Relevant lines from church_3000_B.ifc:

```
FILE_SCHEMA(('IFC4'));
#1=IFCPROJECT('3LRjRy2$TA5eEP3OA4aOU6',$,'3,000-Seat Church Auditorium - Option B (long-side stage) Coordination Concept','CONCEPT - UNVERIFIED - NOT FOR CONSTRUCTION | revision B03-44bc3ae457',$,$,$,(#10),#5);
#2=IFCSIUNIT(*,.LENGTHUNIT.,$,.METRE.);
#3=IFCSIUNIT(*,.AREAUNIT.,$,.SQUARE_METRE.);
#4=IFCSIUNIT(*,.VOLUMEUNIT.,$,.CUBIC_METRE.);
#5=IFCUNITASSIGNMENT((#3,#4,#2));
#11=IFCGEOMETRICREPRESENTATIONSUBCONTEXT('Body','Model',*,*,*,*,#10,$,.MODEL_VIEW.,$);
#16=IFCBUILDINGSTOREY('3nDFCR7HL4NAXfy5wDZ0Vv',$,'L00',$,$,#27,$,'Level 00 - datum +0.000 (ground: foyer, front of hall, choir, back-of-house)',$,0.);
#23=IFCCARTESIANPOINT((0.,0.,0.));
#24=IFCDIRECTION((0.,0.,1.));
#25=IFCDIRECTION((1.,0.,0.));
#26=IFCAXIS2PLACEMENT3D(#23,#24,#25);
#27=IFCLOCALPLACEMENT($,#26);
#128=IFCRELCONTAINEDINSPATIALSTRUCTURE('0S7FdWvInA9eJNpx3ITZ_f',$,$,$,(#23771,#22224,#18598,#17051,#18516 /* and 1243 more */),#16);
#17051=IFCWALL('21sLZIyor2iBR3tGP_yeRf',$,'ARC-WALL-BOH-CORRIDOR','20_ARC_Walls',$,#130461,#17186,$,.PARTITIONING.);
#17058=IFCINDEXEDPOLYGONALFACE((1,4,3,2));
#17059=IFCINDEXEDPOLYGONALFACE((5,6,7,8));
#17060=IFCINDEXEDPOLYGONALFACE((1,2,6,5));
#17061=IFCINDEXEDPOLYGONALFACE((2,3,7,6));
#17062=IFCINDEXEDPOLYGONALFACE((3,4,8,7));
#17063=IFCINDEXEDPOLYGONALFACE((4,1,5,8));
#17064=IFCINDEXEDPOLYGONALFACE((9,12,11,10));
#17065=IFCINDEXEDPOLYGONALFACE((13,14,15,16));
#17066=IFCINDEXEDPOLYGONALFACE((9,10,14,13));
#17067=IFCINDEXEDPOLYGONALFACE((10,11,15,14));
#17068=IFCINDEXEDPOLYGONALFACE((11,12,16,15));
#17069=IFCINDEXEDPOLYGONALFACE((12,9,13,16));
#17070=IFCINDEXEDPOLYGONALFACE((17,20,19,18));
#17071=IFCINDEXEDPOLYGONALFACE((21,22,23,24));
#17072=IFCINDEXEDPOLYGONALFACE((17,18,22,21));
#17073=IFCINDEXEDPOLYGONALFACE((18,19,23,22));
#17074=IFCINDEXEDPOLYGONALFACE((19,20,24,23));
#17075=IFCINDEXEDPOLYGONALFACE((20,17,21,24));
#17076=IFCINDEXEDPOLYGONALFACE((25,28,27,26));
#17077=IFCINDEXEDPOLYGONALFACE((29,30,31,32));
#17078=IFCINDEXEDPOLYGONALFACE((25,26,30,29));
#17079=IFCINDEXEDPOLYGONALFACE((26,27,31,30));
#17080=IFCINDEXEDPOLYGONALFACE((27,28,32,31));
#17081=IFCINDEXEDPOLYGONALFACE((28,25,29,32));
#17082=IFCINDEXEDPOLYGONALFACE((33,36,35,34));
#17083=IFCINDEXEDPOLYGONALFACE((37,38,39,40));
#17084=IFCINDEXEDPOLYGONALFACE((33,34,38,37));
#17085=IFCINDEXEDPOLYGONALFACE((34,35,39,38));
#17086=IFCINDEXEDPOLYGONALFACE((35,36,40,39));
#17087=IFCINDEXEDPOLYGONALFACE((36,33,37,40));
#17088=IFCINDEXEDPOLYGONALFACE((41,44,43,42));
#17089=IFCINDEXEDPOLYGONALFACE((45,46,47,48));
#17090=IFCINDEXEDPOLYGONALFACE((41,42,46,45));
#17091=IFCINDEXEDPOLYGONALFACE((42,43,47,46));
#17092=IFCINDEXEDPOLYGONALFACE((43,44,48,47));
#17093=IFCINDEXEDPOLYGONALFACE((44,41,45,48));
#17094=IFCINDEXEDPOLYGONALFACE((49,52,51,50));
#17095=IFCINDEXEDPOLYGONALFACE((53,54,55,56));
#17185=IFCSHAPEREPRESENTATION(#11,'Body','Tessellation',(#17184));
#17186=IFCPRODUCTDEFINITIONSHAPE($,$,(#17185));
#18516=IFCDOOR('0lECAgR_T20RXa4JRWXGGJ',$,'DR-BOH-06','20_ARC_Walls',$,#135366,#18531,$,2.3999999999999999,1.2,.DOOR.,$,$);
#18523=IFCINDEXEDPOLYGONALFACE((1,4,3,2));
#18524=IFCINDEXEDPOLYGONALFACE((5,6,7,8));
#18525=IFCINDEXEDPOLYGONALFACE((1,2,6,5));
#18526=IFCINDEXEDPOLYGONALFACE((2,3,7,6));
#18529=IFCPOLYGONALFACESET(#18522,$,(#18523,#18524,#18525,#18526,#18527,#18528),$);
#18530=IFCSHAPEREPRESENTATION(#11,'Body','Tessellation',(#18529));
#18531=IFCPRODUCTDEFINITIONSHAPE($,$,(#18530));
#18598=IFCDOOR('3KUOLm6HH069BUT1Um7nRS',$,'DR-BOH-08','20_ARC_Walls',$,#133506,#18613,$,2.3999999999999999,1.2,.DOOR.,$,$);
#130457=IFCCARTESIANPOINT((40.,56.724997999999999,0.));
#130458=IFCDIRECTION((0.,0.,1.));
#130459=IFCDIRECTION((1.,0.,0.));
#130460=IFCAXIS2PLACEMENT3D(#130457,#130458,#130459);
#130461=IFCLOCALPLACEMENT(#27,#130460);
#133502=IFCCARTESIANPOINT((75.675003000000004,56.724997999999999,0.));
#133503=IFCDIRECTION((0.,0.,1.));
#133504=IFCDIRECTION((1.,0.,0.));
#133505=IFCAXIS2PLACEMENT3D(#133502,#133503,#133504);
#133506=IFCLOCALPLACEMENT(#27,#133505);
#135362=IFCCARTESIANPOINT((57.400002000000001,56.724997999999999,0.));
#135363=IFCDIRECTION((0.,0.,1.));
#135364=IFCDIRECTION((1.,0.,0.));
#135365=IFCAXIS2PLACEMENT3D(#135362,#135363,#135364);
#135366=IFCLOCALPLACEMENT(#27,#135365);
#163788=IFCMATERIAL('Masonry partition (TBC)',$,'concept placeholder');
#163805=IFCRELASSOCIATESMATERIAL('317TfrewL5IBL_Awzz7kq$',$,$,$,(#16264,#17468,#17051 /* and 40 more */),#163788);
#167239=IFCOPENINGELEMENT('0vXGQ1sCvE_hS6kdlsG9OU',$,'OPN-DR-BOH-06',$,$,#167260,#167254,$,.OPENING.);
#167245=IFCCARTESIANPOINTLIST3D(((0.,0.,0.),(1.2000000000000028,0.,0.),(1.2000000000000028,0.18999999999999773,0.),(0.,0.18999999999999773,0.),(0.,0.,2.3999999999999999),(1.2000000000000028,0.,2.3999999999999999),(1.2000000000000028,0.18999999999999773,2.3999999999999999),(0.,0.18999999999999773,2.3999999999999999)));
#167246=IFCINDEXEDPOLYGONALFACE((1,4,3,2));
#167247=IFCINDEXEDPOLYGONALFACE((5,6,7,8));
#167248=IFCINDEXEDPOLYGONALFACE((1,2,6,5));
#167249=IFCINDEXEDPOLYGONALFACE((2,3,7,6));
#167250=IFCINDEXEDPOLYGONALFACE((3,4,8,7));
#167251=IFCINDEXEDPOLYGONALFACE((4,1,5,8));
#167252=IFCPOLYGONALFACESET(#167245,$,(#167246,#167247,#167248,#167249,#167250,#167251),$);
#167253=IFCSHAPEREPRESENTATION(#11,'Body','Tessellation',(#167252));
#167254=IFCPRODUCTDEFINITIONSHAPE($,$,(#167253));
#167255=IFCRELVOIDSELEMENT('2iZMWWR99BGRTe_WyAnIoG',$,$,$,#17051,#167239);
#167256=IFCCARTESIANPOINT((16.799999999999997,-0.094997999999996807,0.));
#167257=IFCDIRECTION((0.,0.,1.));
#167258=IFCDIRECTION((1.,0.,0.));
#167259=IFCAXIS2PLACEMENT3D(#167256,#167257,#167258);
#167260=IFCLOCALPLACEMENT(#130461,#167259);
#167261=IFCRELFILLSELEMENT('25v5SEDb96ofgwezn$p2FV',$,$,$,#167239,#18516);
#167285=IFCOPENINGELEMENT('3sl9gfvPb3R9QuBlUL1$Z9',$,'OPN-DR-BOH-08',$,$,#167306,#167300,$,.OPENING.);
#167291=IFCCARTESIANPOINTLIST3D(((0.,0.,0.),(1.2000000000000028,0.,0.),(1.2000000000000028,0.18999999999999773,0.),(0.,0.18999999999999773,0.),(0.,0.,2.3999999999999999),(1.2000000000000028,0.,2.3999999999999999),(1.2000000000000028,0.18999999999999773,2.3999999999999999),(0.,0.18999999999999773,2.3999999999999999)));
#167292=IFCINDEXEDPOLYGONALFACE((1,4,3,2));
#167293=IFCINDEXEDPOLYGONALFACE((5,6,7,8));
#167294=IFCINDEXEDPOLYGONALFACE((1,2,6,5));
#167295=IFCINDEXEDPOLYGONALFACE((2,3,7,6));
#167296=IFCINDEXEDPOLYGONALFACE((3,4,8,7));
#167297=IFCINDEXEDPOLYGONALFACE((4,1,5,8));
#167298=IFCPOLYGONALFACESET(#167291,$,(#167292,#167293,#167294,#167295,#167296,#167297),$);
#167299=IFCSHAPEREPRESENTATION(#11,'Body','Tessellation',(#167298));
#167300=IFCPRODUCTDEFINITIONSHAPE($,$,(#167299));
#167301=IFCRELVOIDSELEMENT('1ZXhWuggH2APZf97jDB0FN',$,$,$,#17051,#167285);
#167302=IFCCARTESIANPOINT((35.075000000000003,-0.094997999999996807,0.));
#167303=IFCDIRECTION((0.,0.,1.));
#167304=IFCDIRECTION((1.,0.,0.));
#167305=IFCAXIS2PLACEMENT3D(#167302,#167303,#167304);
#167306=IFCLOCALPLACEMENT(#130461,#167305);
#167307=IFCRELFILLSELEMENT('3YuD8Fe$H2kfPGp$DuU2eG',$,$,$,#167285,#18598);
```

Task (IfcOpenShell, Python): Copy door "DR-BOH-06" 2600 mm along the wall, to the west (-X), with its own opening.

```python
import ifcopenshell
import ifcopenshell.api.feature
import ifcopenshell.api.geometry
import ifcopenshell.api.root
import ifcopenshell.geom
import ifcopenshell.util.element
import ifcopenshell.util.placement
import ifcopenshell.util.shape
import ifcopenshell.util.unit

model = ifcopenshell.open("church_3000_B.ifc")
unit_scale = ifcopenshell.util.unit.calculate_unit_scale(model)
settings = ifcopenshell.geom.settings()


def volume(element):
    """Net volume in cubic metres, openings subtracted."""
    shape = ifcopenshell.geom.create_shape(settings, element)
    return ifcopenshell.util.shape.get_volume(shape.geometry)


door = model.by_guid("0lECAgR_T20RXa4JRWXGGJ")
opening = door.FillsVoids[0].RelatingOpeningElement
wall = opening.VoidsElements[0].RelatingBuildingElement
before = volume(wall)
shift = ifcopenshell.util.placement.get_local_placement(wall.ObjectPlacement)[:3, 0] * -2.6 / unit_scale

# copy_class copies the void relationship, type, container and properties, but no geometry.
new_opening = ifcopenshell.api.root.copy_class(model, product=opening)
new_opening.Representation = ifcopenshell.util.element.copy_deep(
    model, opening.Representation, exclude=["IfcGeometricRepresentationContext", "IfcRepresentationMap"]
)
new_door = ifcopenshell.api.root.copy_class(model, product=door)
new_door.Representation = ifcopenshell.util.element.copy_deep(
    model, door.Representation, exclude=["IfcGeometricRepresentationContext", "IfcRepresentationMap"]
)
ifcopenshell.api.feature.add_filling(model, opening=new_opening, element=new_door)

for old, new in ((opening, new_opening), (door, new_door)):
    matrix = ifcopenshell.util.placement.get_local_placement(old.ObjectPlacement)
    matrix[:3, 3] += shift
    ifcopenshell.api.geometry.edit_object_placement(model, product=new, matrix=matrix, is_si=False)

after = volume(wall)

print(f"wall volume {before:.3f} -> {after:.3f} m3")

model.write("church_3000_B_rev.ifc")
```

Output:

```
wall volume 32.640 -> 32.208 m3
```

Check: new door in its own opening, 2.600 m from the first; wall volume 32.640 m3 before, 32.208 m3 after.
